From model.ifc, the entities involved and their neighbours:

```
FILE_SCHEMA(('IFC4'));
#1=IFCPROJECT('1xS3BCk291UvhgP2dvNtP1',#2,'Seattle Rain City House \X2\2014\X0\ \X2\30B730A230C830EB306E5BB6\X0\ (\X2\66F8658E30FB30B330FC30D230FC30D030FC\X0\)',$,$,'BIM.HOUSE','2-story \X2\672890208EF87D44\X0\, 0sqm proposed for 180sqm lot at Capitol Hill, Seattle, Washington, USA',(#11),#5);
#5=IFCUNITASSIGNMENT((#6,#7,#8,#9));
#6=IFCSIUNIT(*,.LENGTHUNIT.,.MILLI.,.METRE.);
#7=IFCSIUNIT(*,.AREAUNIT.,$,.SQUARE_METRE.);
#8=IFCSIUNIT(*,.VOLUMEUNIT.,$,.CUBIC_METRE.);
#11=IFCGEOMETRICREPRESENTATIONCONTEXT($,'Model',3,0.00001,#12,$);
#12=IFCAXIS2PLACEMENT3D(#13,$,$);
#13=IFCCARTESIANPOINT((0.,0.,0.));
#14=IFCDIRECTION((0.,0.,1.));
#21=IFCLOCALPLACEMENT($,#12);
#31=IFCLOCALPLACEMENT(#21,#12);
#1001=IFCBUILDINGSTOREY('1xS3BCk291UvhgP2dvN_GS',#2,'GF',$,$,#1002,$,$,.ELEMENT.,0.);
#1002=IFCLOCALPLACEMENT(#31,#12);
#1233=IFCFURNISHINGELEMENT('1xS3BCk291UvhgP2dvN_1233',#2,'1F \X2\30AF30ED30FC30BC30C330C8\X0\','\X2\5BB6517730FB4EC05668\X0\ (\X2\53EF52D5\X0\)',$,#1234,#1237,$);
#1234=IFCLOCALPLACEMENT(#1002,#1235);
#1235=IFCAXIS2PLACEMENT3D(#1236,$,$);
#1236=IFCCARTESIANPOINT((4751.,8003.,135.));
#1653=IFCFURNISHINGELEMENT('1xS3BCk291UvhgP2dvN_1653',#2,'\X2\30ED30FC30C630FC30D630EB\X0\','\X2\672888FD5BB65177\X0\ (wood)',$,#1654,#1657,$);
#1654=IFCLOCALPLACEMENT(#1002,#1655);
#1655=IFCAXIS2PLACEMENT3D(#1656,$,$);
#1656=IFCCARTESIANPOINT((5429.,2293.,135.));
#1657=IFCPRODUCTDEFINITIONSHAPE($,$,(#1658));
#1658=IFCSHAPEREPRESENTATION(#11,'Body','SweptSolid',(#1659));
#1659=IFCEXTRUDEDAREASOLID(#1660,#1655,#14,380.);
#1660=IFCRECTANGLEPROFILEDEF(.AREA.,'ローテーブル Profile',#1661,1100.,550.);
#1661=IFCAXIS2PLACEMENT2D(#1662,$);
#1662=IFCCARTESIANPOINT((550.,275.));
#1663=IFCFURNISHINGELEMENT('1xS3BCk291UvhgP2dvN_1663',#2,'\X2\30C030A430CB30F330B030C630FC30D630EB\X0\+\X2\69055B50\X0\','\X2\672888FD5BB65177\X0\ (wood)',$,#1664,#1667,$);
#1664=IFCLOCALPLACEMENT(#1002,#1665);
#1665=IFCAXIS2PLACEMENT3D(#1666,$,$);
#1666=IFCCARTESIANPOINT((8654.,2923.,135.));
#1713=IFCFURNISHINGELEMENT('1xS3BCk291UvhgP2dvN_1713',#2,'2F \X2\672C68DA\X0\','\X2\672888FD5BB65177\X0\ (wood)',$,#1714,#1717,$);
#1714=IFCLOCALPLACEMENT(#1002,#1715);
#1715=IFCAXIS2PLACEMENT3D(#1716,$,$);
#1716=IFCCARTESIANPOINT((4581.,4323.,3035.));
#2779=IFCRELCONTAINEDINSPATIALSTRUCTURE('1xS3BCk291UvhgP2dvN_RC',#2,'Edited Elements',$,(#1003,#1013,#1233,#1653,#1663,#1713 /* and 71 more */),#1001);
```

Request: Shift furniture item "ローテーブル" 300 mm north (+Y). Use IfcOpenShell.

```python
import ifcopenshell
import ifcopenshell.api.geometry
import ifcopenshell.util.placement
import ifcopenshell.util.unit

model = ifcopenshell.open("model.ifc")
unit_scale = ifcopenshell.util.unit.calculate_unit_scale(model)

item = model.by_guid("1xS3BCk291UvhgP2dvN_1653")
matrix = ifcopenshell.util.placement.get_local_placement(item.ObjectPlacement)
matrix[1, 3] += 0.3 / unit_scale
ifcopenshell.api.geometry.edit_object_placement(model, product=item, matrix=matrix, is_si=False)

print(ifcopenshell.util.placement.get_local_placement(item.ObjectPlacement).round(3) + 0.0)

model.write("model-out.ifc")
```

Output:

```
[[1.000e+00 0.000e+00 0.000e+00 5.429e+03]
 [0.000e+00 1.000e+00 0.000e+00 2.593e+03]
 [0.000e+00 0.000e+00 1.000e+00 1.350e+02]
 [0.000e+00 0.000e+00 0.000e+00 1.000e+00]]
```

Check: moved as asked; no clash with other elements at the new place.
